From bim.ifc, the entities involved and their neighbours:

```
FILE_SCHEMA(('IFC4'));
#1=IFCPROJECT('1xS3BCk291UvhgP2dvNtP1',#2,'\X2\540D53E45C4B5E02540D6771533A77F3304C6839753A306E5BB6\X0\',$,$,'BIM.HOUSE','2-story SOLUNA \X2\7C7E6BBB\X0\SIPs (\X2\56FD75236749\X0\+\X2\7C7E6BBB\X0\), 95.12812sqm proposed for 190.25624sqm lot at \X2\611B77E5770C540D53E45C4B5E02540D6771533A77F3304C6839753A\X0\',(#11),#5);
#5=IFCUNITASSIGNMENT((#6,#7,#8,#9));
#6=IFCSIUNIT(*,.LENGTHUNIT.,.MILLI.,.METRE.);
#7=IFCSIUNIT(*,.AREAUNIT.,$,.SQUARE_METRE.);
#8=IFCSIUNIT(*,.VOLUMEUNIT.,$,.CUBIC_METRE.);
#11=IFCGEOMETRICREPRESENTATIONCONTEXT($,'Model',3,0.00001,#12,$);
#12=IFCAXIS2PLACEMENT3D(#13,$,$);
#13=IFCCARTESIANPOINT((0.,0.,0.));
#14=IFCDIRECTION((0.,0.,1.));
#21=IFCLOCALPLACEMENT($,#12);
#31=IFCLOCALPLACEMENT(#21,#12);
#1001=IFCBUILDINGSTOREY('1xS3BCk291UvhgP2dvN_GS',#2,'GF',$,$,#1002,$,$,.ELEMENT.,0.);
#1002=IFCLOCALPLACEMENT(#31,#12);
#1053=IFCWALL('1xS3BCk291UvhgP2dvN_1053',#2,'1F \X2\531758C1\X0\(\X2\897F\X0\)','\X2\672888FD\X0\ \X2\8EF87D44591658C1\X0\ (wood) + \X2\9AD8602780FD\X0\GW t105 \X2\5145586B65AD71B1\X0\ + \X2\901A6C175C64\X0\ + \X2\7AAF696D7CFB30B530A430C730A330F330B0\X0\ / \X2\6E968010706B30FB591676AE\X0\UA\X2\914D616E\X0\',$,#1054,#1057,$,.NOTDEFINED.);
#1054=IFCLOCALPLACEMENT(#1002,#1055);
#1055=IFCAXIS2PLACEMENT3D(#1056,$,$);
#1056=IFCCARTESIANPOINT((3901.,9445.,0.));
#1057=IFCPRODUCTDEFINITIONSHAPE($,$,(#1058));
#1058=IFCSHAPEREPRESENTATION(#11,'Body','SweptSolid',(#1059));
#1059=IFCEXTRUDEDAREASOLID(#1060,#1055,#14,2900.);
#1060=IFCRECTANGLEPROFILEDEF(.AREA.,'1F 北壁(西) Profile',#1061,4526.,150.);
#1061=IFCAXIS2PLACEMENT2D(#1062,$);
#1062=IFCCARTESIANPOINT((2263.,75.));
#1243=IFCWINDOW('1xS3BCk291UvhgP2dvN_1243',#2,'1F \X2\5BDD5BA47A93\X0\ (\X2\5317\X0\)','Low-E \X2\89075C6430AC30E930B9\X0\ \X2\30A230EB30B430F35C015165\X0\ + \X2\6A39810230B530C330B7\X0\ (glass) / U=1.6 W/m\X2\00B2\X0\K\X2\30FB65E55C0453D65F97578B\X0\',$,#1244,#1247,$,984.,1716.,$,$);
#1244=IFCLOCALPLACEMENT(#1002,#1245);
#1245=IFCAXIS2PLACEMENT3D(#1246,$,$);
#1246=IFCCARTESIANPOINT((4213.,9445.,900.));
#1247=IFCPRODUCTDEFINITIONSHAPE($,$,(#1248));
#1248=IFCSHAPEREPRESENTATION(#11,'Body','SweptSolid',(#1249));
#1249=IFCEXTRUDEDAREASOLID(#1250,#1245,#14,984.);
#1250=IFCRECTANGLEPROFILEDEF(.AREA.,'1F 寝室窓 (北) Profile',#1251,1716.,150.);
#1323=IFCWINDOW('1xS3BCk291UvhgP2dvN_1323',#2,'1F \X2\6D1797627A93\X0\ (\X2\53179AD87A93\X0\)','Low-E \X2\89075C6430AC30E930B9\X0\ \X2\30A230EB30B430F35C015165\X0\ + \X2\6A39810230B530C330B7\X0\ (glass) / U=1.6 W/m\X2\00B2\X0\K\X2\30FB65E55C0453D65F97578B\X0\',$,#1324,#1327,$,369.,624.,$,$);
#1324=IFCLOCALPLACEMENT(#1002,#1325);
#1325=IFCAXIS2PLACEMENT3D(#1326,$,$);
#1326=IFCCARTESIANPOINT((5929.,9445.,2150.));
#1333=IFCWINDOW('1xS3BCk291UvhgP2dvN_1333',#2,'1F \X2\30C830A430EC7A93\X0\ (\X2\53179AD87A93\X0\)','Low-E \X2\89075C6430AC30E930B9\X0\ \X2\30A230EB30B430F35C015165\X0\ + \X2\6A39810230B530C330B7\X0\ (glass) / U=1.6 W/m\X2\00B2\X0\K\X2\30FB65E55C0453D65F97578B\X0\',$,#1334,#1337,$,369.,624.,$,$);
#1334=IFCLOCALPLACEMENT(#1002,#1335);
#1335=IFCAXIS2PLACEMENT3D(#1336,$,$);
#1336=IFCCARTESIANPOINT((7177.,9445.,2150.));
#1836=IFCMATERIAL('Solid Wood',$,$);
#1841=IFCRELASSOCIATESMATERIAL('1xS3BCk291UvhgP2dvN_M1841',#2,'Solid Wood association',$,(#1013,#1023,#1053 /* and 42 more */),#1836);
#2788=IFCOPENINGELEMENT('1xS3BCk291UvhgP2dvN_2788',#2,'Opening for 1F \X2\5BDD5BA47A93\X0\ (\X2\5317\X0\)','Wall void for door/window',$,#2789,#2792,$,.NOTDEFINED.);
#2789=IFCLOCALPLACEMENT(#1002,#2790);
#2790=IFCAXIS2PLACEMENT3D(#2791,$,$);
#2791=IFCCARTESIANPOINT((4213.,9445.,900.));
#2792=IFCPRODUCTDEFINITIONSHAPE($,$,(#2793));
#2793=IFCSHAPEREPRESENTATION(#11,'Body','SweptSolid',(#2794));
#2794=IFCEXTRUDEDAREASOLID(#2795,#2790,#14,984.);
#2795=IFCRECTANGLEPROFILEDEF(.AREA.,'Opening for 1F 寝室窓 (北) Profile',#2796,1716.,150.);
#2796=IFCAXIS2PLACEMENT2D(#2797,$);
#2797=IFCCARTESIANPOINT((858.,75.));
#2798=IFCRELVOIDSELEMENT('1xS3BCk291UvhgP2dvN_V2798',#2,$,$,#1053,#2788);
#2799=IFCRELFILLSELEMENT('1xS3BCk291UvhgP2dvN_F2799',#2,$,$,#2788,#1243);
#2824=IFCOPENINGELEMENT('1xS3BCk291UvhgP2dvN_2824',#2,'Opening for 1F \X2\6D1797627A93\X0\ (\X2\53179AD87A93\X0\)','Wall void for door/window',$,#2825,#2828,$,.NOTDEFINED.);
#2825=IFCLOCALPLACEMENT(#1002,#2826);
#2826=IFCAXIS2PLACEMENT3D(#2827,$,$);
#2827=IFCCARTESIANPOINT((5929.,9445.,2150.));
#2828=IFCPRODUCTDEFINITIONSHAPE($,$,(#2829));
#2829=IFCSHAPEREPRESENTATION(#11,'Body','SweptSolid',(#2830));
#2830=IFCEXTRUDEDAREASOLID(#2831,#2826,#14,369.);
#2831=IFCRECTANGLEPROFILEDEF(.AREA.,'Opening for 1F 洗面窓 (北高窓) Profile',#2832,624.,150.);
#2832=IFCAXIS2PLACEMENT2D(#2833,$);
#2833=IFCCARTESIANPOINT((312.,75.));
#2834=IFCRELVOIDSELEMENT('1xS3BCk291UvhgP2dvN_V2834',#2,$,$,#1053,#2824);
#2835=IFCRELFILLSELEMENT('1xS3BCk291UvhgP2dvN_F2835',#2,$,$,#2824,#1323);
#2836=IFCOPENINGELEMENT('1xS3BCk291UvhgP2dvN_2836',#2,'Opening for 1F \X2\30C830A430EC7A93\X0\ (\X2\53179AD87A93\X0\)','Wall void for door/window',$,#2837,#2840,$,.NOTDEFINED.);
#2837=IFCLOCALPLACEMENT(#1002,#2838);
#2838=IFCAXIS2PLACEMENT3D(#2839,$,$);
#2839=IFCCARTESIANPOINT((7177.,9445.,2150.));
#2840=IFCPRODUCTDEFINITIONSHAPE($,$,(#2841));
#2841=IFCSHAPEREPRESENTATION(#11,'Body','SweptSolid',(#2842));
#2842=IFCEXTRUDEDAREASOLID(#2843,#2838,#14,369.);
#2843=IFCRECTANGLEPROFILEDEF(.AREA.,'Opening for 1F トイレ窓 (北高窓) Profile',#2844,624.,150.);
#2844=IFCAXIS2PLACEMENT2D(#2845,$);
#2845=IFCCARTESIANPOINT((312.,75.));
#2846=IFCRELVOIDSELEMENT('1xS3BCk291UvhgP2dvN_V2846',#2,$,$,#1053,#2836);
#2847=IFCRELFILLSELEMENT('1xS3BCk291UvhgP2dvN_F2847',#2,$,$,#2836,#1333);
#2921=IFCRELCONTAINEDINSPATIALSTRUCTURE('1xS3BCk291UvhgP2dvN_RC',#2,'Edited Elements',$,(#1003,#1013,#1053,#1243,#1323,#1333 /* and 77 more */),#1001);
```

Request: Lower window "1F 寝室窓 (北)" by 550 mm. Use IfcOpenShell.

```python
import numpy as np
import ifcopenshell
import ifcopenshell.api.geometry
import ifcopenshell.util.placement
import ifcopenshell.util.unit

model = ifcopenshell.open("bim.ifc")
unit_scale = ifcopenshell.util.unit.calculate_unit_scale(model)

window = model.by_guid("1xS3BCk291UvhgP2dvN_1243")
opening = window.FillsVoids[0].RelatingOpeningElement
dz = -550.0

shift = np.array([0.0, 0.0, dz])
# The window is not placed relative to its opening, so move both.
for product in (opening, window):
    matrix = ifcopenshell.util.placement.get_local_placement(product.ObjectPlacement)
    matrix[:3, 3] += shift
    ifcopenshell.api.geometry.edit_object_placement(model, product=product, matrix=matrix, is_si=False)

print(f"moved by {dz * unit_scale:+.3f} m")

model.write("bim_updated.ifc")
```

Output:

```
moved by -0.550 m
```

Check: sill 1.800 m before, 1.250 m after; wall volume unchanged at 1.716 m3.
